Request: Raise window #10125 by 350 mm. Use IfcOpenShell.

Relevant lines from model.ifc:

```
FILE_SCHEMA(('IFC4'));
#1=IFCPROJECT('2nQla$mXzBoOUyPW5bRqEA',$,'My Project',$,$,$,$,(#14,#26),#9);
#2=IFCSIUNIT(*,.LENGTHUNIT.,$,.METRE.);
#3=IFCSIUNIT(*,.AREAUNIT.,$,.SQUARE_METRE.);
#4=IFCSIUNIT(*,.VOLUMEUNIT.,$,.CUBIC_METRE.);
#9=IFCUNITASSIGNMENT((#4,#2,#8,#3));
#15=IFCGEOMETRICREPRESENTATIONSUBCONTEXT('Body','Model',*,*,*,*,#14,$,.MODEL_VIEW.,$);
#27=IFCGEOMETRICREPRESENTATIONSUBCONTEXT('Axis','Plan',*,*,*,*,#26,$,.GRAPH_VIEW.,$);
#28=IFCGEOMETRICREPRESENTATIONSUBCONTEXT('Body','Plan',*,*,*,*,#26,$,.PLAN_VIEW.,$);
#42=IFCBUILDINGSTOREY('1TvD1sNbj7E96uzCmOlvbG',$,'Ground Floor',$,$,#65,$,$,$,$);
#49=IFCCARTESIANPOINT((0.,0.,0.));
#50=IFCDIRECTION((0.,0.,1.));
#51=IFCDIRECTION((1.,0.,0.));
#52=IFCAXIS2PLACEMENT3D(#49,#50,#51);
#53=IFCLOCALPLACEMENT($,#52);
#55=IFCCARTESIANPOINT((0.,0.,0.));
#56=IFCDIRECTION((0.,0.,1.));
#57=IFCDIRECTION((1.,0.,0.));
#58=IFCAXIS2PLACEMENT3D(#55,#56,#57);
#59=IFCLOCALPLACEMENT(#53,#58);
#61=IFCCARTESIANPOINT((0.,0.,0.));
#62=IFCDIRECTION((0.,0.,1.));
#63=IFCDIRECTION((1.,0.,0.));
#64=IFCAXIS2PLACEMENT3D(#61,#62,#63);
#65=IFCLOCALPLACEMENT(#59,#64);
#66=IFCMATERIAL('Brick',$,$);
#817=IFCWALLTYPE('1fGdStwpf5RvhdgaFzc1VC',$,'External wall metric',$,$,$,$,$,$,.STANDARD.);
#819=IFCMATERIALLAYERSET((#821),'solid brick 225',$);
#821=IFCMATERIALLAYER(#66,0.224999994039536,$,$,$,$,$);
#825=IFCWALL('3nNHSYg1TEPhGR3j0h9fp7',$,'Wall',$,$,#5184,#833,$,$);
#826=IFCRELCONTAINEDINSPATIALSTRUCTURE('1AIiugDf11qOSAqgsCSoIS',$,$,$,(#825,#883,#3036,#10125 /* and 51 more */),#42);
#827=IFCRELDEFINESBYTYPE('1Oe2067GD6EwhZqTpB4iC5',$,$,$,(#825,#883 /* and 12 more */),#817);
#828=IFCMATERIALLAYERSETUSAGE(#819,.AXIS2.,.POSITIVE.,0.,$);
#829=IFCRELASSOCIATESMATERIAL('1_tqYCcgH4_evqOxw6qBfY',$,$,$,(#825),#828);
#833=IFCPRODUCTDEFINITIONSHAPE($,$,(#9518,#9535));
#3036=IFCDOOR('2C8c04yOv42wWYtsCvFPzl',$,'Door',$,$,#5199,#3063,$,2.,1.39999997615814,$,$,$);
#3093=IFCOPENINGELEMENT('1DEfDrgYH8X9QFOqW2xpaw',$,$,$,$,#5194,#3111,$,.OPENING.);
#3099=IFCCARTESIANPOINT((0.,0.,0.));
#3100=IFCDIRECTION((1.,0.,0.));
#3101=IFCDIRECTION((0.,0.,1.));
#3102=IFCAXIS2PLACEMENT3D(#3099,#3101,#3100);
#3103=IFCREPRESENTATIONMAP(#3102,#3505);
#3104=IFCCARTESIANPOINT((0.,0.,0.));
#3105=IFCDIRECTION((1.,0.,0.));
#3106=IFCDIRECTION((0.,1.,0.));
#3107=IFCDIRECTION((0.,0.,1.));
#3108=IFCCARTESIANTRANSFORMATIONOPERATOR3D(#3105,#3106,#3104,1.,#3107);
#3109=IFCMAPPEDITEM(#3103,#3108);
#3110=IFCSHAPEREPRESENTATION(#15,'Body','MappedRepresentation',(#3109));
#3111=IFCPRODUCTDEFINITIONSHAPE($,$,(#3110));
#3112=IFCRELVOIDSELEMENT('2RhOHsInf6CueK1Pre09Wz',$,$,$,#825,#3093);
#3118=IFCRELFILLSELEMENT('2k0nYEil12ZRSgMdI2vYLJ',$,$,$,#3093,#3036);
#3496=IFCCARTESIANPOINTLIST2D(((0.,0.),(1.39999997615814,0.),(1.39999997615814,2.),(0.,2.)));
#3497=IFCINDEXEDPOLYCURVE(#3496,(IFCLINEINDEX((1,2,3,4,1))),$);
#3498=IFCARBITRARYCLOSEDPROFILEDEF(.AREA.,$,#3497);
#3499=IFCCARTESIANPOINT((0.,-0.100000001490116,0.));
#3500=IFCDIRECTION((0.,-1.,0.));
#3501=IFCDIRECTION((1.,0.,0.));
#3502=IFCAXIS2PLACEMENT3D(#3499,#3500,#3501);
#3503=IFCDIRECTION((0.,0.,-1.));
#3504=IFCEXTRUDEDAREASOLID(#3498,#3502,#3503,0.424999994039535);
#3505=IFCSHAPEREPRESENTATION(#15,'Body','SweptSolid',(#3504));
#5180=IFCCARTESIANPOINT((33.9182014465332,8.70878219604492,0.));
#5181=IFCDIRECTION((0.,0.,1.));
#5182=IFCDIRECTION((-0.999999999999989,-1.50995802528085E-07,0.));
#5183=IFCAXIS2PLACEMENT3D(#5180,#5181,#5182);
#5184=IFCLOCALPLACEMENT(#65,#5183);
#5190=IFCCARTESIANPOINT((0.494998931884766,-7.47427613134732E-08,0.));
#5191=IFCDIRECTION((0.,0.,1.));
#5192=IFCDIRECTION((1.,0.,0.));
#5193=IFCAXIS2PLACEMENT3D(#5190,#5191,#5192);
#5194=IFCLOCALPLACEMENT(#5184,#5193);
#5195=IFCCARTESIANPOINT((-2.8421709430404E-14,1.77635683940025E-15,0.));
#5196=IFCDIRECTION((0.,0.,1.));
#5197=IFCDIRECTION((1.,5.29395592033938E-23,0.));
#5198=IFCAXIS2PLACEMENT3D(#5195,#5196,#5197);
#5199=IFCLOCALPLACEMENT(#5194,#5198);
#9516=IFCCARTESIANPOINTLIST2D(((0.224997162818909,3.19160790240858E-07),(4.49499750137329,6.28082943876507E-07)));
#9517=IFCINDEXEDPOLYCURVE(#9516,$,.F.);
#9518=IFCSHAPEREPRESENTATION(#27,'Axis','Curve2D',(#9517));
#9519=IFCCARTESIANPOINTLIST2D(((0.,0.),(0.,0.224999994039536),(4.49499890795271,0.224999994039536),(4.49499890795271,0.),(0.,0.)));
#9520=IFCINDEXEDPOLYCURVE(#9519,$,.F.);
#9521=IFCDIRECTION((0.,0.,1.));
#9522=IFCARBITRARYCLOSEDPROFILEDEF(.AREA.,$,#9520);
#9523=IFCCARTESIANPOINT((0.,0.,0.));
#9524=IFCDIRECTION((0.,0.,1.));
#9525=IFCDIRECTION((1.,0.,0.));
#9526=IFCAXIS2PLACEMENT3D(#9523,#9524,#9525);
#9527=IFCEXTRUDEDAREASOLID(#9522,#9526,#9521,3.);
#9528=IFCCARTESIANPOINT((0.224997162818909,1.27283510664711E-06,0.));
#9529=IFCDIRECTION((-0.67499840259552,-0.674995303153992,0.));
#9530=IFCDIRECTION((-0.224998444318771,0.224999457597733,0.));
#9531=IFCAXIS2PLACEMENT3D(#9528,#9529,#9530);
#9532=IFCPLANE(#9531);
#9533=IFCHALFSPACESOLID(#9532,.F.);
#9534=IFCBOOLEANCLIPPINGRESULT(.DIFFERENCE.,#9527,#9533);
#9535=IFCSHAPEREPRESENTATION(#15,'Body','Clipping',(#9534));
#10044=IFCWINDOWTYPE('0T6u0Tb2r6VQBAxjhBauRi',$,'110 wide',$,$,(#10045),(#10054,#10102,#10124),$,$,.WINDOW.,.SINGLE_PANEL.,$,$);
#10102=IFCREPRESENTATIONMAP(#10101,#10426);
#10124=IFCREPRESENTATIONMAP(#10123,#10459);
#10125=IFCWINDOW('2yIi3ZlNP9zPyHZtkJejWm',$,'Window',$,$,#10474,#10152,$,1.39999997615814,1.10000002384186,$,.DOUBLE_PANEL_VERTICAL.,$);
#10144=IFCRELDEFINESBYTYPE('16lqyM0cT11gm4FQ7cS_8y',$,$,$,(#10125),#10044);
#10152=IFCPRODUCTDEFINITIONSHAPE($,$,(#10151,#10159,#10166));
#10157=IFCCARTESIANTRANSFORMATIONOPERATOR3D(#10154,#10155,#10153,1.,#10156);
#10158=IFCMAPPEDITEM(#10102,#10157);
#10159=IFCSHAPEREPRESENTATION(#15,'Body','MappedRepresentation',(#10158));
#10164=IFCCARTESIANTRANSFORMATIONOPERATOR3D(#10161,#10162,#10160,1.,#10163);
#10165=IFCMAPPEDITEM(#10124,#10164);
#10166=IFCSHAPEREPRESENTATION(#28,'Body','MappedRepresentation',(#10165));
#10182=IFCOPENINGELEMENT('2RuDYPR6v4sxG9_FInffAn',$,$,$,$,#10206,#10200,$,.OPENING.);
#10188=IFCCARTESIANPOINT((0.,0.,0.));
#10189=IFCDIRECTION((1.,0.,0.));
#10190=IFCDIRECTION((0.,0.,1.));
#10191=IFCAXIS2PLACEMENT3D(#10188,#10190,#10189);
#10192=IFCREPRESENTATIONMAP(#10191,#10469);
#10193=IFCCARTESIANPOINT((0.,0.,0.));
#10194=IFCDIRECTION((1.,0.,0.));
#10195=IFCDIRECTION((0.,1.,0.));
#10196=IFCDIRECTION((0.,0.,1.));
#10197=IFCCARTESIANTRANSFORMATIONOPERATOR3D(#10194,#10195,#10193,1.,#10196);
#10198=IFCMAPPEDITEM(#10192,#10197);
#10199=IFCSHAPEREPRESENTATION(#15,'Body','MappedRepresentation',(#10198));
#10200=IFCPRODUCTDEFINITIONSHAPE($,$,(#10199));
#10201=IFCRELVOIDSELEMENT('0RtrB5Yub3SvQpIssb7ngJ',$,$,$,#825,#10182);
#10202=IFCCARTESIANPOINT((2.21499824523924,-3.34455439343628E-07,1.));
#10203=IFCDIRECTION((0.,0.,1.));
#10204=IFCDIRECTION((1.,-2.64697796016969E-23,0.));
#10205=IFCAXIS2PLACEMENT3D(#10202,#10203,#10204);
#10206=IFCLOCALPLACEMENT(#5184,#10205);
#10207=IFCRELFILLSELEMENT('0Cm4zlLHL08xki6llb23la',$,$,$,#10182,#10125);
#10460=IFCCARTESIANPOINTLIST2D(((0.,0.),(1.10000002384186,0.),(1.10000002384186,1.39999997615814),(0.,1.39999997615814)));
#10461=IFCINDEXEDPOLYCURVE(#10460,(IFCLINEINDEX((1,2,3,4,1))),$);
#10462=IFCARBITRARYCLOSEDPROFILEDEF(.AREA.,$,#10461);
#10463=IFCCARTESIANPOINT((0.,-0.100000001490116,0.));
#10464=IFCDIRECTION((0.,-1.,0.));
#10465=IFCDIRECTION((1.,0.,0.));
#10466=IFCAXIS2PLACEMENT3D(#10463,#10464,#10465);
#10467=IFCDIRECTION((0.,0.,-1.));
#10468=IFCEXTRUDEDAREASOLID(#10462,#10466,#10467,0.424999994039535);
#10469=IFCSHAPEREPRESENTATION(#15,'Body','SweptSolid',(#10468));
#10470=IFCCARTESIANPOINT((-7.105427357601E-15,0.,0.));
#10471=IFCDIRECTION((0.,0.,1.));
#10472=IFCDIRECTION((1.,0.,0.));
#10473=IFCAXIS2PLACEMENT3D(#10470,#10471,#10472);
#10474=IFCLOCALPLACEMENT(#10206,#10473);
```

```python
import numpy as np
import ifcopenshell
import ifcopenshell.api.geometry
import ifcopenshell.util.placement
import ifcopenshell.util.unit

model = ifcopenshell.open("model.ifc")
unit_scale = ifcopenshell.util.unit.calculate_unit_scale(model)

window = model.by_guid("2yIi3ZlNP9zPyHZtkJejWm")
opening = window.FillsVoids[0].RelatingOpeningElement
dz = 0.35

shift = np.array([0.0, 0.0, dz])
# The window is placed relative to its opening, so it follows when the opening moves.
matrix = ifcopenshell.util.placement.get_local_placement(opening.ObjectPlacement)
matrix[:3, 3] += shift
ifcopenshell.api.geometry.edit_object_placement(
    model, product=opening, matrix=matrix, is_si=False, should_transform_children=True
)

print(f"moved by {dz * unit_scale:+.3f} m")

model.write("model_rev.ifc")
```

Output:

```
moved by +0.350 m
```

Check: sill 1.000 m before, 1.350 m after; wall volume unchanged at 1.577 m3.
